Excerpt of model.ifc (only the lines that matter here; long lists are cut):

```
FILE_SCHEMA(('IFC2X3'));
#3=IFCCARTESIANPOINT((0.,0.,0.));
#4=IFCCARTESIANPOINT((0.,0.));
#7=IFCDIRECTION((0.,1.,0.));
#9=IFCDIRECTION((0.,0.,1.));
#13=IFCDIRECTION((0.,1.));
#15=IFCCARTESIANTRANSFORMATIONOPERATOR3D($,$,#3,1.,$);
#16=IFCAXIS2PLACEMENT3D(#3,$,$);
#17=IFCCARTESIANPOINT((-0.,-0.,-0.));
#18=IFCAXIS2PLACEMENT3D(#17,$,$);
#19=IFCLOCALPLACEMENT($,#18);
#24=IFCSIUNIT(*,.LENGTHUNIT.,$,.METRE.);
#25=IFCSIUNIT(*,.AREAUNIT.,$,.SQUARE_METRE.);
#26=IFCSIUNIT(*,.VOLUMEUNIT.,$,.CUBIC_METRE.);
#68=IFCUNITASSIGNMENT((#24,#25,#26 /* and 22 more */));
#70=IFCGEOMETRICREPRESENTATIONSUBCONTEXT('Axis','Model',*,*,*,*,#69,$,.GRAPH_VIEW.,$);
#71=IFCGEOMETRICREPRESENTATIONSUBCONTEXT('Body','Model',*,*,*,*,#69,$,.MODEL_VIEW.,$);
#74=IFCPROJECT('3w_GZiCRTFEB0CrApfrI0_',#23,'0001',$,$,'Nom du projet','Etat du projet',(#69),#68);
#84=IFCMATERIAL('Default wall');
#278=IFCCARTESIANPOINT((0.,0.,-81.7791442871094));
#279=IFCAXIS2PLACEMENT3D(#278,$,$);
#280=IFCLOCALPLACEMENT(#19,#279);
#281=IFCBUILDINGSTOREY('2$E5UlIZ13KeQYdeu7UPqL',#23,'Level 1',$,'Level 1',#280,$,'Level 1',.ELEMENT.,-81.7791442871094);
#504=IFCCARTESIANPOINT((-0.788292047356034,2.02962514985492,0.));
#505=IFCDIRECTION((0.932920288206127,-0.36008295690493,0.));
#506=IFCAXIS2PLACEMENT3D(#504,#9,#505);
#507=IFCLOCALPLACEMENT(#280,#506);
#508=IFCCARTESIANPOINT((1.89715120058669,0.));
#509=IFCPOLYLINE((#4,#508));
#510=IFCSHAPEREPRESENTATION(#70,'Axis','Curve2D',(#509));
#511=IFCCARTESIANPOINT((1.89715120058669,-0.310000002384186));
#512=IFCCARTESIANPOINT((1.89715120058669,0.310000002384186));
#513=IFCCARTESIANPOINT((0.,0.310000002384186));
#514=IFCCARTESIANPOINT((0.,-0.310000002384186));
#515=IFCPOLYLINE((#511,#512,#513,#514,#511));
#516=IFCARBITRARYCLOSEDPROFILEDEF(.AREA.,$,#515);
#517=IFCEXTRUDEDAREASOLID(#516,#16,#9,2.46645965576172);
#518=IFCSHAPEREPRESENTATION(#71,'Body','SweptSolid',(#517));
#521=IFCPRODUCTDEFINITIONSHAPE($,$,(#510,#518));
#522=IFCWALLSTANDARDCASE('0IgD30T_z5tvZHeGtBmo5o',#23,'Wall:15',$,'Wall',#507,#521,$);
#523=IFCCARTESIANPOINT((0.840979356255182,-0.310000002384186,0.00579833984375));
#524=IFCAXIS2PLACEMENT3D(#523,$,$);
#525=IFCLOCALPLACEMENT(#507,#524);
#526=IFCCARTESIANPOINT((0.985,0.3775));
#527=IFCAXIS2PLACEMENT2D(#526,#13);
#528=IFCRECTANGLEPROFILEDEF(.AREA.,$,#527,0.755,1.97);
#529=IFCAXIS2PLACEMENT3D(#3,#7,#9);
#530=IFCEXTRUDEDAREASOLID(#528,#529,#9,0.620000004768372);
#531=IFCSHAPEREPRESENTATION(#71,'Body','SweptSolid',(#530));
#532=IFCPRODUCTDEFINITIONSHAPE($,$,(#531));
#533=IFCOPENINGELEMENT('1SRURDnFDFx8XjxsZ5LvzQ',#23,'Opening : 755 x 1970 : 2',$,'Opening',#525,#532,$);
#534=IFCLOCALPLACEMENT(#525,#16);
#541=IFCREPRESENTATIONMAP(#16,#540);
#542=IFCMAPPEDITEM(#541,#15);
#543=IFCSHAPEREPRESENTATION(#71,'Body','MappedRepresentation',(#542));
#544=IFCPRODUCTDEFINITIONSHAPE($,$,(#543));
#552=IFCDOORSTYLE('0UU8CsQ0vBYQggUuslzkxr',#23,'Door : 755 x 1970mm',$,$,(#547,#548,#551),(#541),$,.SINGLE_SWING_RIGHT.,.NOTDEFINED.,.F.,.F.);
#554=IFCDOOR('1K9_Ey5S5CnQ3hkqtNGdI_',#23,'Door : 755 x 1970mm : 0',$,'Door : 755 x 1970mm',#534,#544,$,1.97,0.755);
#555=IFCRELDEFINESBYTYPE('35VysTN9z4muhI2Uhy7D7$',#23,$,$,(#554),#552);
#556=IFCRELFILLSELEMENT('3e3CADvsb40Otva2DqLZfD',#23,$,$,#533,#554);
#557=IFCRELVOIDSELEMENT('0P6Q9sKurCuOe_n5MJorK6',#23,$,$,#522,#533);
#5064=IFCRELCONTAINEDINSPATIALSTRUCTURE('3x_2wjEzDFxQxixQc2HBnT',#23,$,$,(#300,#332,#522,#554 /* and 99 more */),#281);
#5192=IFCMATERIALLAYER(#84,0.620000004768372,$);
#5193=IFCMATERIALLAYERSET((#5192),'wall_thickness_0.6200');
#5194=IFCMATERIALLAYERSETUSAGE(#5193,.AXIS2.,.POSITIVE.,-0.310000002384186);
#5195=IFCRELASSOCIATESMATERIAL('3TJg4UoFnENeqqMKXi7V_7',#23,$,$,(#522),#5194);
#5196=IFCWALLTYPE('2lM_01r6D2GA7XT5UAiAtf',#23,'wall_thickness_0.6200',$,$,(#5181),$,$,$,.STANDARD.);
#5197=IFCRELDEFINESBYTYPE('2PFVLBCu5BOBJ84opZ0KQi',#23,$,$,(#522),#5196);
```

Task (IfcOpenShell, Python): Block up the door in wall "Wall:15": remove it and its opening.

```python
import ifcopenshell
import ifcopenshell.api.feature
import ifcopenshell.api.root
import ifcopenshell.geom
import ifcopenshell.util.shape

model = ifcopenshell.open("model.ifc")
settings = ifcopenshell.geom.settings()


def volume(element):
    """Net volume in cubic metres, openings subtracted."""
    shape = ifcopenshell.geom.create_shape(settings, element)
    return ifcopenshell.util.shape.get_volume(shape.geometry)


door = model.by_guid("1K9_Ey5S5CnQ3hkqtNGdI_")
opening = door.FillsVoids[0].RelatingOpeningElement
wall = opening.VoidsElements[0].RelatingBuildingElement
before = volume(wall)

ifcopenshell.api.root.remove_product(model, product=door)
ifcopenshell.api.feature.remove_feature(model, feature=opening)

after = volume(wall)

print(f"wall volume {before:.3f} -> {after:.3f} m3")

model.write("model_rev.ifc")
```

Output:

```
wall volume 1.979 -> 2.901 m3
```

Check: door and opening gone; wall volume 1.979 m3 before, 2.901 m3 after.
